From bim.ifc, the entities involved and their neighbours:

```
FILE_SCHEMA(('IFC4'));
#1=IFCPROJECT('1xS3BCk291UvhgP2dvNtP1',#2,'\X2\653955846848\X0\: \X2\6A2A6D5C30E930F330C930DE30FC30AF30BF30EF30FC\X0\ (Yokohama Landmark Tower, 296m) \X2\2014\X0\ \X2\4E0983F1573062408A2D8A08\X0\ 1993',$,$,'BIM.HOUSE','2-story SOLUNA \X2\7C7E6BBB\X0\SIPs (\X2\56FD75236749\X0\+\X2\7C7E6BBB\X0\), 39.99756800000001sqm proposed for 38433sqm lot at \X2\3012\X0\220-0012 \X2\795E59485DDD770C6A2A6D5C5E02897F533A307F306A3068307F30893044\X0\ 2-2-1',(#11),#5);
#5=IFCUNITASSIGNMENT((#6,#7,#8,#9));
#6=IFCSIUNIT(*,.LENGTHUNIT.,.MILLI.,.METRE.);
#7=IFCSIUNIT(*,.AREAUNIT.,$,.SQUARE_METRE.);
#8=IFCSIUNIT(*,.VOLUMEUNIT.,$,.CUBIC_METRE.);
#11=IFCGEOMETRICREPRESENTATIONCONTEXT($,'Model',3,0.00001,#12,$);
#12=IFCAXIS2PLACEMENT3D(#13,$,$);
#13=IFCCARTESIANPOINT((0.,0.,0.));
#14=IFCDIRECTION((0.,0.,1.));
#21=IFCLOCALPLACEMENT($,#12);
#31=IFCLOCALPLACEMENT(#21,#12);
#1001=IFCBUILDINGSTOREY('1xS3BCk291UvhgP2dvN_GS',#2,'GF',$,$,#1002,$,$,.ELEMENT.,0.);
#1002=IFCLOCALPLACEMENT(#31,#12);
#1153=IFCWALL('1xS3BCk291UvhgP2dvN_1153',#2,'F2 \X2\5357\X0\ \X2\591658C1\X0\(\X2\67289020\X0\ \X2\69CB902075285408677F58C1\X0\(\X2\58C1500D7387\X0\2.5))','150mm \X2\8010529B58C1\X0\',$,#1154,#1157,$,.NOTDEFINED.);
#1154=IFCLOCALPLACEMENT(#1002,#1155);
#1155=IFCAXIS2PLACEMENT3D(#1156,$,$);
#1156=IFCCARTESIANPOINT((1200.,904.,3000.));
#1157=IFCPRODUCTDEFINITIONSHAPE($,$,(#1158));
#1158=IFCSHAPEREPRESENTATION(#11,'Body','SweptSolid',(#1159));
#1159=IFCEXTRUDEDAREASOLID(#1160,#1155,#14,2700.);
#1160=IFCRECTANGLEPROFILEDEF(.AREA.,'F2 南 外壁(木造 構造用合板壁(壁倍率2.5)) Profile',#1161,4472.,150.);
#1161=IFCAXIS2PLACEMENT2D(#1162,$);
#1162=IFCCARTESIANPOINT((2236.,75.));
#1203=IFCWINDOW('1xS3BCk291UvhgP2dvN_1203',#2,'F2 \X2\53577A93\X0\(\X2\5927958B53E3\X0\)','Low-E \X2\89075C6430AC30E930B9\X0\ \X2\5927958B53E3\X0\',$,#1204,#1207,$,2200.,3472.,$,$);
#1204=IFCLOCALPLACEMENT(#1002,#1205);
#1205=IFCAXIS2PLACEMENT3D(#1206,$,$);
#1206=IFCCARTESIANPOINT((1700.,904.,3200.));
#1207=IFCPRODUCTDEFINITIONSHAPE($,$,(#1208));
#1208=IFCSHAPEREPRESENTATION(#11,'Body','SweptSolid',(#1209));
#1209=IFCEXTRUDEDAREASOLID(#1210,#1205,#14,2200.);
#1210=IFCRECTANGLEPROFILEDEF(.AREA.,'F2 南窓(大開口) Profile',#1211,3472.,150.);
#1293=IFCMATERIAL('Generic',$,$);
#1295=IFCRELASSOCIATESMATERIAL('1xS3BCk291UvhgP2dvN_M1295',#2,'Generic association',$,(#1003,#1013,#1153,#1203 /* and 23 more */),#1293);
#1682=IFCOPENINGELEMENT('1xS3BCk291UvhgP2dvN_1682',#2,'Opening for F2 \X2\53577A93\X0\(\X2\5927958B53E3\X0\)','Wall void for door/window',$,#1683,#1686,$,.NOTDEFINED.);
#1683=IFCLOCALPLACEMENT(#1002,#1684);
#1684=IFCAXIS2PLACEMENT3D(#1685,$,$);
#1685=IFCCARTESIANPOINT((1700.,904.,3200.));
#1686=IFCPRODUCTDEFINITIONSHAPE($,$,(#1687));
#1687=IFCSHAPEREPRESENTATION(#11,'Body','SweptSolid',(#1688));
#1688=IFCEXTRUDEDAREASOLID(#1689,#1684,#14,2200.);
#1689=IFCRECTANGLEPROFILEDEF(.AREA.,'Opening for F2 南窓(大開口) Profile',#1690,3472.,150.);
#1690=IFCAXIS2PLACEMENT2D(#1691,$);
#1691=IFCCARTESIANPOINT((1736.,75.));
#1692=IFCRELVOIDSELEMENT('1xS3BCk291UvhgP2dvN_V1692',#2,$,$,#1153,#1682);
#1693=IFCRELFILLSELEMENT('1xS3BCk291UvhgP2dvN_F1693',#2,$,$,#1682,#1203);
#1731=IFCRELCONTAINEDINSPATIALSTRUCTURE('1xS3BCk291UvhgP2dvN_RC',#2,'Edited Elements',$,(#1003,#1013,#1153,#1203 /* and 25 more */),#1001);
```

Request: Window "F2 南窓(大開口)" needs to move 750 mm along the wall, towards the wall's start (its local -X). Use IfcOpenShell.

```python
import ifcopenshell
import ifcopenshell.api.geometry
import ifcopenshell.util.placement

model = ifcopenshell.open("bim.ifc")

window = model.by_guid("1xS3BCk291UvhgP2dvN_1203")
opening = window.FillsVoids[0].RelatingOpeningElement
wall = opening.VoidsElements[0].RelatingBuildingElement

wall_matrix = ifcopenshell.util.placement.get_local_placement(wall.ObjectPlacement)
shift = wall_matrix[:3, 0] * -750.0
before = ifcopenshell.util.placement.get_local_placement(window.ObjectPlacement)[:3, 3].copy()

# The window is not placed relative to its opening, so move both.
for product in (opening, window):
    matrix = ifcopenshell.util.placement.get_local_placement(product.ObjectPlacement)
    matrix[:3, 3] += shift
    ifcopenshell.api.geometry.edit_object_placement(model, product=product, matrix=matrix, is_si=False)

after = ifcopenshell.util.placement.get_local_placement(window.ObjectPlacement)[:3, 3]
print("window moved by", (after - before).round(3) + 0.0)

model.write("bim-out.ifc")
```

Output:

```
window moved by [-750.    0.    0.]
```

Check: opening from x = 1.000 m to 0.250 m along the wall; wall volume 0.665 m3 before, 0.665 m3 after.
